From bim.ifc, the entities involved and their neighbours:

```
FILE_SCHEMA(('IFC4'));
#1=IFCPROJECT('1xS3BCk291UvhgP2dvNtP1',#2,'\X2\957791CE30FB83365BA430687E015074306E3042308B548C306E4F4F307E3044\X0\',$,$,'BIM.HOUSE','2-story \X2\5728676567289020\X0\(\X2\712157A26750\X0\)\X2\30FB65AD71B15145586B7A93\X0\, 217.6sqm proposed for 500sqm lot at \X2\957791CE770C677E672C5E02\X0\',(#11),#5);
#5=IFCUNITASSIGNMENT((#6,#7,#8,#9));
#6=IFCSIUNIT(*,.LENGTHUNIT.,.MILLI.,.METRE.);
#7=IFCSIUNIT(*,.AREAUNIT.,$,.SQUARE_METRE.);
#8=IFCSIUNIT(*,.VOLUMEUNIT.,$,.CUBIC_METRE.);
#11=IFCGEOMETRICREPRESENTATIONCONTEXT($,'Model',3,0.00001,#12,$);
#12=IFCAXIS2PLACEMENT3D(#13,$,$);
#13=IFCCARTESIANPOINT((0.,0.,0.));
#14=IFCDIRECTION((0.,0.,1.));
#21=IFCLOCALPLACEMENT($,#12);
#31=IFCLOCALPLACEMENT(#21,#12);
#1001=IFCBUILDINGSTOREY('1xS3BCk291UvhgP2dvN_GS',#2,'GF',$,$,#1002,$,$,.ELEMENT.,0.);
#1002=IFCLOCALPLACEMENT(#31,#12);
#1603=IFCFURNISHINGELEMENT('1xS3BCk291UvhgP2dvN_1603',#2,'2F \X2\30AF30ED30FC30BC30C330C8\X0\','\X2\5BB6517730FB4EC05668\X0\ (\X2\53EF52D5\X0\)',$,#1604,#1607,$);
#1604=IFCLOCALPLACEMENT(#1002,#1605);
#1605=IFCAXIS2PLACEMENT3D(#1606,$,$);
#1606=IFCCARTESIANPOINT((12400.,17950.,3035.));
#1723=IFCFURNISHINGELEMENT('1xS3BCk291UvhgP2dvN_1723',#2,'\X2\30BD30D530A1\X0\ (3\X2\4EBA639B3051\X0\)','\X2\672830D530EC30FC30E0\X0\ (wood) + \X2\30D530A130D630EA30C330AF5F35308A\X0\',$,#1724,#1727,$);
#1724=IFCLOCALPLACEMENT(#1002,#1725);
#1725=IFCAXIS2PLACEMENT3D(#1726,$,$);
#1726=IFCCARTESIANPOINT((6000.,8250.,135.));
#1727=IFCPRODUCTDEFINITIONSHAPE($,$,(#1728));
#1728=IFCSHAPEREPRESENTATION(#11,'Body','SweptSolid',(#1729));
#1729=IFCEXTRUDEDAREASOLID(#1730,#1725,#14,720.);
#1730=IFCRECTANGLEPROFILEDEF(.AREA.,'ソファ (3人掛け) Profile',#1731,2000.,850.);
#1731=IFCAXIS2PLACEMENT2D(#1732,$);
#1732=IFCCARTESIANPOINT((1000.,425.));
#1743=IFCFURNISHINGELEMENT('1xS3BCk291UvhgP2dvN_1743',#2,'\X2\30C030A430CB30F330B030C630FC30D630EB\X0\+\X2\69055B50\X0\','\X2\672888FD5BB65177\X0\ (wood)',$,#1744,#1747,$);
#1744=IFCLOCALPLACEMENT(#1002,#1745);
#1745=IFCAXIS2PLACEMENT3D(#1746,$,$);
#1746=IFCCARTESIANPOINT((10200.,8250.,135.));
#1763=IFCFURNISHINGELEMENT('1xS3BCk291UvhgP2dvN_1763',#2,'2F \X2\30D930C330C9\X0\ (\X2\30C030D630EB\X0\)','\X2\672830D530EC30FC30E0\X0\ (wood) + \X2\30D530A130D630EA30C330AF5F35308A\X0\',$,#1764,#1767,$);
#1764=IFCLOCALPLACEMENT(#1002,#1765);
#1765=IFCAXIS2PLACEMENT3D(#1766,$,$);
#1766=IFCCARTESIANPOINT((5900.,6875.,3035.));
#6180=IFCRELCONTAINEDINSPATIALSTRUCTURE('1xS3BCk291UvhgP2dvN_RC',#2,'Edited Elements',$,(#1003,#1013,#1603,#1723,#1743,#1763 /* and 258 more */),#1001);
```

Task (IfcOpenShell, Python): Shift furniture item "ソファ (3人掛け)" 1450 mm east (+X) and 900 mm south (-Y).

```python
import ifcopenshell
import ifcopenshell.api.geometry
import ifcopenshell.util.placement
import ifcopenshell.util.unit

model = ifcopenshell.open("bim.ifc")
unit_scale = ifcopenshell.util.unit.calculate_unit_scale(model)

item = model.by_id(1723)
matrix = ifcopenshell.util.placement.get_local_placement(item.ObjectPlacement)
matrix[0, 3] += 1.45 / unit_scale
matrix[1, 3] -= 0.9 / unit_scale
ifcopenshell.api.geometry.edit_object_placement(model, product=item, matrix=matrix, is_si=False)

print(ifcopenshell.util.placement.get_local_placement(item.ObjectPlacement).round(3) + 0.0)

model.write("bim-out.ifc")
```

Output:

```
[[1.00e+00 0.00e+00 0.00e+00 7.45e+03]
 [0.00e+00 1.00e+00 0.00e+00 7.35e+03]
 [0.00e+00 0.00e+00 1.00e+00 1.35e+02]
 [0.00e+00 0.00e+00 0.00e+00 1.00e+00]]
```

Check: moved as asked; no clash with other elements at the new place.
